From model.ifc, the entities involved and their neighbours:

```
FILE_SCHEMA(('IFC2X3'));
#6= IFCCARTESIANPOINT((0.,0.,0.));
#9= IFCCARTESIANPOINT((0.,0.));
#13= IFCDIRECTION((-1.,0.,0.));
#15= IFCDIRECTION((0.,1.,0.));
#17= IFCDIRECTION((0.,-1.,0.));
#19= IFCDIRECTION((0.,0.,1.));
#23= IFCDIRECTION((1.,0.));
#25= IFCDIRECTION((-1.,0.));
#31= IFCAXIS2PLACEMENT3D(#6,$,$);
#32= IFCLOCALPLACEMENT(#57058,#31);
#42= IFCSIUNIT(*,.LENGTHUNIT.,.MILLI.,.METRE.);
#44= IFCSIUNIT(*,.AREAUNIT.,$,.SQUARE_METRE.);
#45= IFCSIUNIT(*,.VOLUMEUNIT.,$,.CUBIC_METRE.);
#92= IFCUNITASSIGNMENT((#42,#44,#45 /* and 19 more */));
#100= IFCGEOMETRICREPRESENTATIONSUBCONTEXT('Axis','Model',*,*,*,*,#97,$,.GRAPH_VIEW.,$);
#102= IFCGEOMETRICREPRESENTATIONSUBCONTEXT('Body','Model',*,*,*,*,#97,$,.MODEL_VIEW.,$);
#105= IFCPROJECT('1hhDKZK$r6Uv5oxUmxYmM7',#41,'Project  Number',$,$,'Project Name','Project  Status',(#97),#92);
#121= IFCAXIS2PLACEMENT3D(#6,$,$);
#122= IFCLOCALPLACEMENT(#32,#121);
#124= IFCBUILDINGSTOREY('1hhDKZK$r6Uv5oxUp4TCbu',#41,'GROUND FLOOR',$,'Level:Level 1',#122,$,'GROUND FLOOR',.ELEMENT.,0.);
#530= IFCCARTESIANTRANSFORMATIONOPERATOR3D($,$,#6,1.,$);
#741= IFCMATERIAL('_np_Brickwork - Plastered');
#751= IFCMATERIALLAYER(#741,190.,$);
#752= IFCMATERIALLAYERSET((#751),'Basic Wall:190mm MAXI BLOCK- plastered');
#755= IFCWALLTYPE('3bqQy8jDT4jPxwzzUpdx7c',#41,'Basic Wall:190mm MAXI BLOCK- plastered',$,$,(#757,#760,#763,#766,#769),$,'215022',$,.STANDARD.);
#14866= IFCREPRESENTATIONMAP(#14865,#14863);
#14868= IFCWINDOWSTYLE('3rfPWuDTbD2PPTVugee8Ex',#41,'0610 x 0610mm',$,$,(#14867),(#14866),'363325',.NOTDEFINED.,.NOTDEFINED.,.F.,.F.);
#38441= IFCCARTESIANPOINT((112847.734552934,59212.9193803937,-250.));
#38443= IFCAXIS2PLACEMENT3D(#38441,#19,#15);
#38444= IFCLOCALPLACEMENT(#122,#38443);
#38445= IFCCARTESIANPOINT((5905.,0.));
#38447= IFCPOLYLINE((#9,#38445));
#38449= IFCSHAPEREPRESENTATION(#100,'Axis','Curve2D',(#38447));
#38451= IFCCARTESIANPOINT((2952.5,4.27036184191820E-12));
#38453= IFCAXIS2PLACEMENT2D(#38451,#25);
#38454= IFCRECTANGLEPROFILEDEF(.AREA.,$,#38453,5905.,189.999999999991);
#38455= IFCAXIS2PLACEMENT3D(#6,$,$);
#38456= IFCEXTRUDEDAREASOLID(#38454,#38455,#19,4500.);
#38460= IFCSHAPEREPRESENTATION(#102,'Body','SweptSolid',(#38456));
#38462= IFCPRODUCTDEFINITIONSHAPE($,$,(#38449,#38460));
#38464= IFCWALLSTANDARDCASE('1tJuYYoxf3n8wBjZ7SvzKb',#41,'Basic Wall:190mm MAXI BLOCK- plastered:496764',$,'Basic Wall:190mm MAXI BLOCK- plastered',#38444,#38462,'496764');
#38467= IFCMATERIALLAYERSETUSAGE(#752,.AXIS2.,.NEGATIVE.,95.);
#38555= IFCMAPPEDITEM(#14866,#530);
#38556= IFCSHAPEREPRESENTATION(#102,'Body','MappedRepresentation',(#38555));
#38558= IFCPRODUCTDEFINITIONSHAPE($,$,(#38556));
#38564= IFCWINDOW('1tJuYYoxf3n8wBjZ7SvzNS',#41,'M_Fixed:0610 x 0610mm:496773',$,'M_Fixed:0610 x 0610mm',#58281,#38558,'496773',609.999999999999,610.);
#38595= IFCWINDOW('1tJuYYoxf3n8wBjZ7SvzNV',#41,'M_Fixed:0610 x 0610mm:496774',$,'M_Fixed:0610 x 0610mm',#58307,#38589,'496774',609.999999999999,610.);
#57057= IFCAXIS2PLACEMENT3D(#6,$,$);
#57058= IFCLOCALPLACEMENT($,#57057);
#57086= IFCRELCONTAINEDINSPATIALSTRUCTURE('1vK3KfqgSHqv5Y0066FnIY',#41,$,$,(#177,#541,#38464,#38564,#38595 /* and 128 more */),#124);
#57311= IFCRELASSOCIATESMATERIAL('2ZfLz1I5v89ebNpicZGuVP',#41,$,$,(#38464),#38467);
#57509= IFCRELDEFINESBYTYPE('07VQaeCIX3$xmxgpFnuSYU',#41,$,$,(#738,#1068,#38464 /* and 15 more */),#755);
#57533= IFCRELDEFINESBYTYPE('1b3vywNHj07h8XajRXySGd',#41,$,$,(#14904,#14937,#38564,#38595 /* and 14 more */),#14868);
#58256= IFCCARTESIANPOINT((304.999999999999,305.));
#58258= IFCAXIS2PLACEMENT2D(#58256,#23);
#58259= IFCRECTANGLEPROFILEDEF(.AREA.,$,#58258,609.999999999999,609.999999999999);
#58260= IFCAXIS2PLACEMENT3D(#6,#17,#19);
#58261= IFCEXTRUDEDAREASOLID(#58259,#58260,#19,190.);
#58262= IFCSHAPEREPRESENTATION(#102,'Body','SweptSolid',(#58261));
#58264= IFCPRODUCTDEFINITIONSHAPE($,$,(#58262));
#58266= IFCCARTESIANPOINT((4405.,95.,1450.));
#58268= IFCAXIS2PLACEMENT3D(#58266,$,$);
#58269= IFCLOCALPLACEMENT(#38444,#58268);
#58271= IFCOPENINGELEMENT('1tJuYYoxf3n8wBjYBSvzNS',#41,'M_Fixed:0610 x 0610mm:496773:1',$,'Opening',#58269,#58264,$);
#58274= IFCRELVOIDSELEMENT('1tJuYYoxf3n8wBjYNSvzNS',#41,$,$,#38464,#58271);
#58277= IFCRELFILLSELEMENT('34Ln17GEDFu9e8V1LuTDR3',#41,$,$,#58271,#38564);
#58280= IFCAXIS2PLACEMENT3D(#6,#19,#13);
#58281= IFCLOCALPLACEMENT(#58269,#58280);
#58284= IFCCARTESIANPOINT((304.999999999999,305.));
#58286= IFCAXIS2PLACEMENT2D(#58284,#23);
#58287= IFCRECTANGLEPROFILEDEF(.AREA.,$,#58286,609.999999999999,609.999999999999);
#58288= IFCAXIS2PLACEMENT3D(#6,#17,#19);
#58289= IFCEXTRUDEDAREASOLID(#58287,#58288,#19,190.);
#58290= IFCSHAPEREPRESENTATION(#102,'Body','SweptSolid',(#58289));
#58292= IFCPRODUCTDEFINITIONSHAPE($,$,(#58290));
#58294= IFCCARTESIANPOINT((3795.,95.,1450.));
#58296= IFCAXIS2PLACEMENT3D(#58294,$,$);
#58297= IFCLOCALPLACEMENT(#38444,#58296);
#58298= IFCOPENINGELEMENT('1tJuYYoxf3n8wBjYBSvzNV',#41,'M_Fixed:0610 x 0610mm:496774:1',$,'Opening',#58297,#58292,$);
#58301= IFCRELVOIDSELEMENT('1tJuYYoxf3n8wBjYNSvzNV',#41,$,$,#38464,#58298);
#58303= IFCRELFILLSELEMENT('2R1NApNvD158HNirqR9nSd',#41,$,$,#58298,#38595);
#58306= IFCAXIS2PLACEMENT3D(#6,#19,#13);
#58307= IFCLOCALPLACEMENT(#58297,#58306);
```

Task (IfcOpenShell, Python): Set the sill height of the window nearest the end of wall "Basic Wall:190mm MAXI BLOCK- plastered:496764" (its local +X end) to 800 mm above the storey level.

```python
import numpy as np
import ifcopenshell
import ifcopenshell.api.geometry
import ifcopenshell.geom
import ifcopenshell.util.element
import ifcopenshell.util.placement
import ifcopenshell.util.shape
import ifcopenshell.util.unit

model = ifcopenshell.open("model.ifc")
unit_scale = ifcopenshell.util.unit.calculate_unit_scale(model)

window = model.by_guid("1tJuYYoxf3n8wBjZ7SvzNS")
opening = window.FillsVoids[0].RelatingOpeningElement
storey = ifcopenshell.util.element.get_container(window, ifc_class="IfcBuildingStorey")
level = ifcopenshell.util.placement.get_local_placement(storey.ObjectPlacement)[2, 3]

# The opening's origin need not be at the sill, so measure its lowest point.
shape = ifcopenshell.geom.create_shape(ifcopenshell.geom.settings(), opening)
bottom = ifcopenshell.util.shape.get_shape_bottom_elevation(shape, shape.geometry) / unit_scale
dz = level + 0.8 / unit_scale - bottom

shift = np.array([0.0, 0.0, dz])
# The window is placed relative to its opening, so it follows when the opening moves.
matrix = ifcopenshell.util.placement.get_local_placement(opening.ObjectPlacement)
matrix[:3, 3] += shift
ifcopenshell.api.geometry.edit_object_placement(
    model, product=opening, matrix=matrix, is_si=False, should_transform_children=True
)

print(f"moved by {dz * unit_scale:+.3f} m")

model.write("model_updated.ifc")
```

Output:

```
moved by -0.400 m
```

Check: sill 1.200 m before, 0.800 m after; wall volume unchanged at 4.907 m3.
